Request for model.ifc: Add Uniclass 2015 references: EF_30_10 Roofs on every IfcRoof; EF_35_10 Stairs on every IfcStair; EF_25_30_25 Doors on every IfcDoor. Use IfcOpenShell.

First a look at what the model holds.

```python
import ifcopenshell

model = ifcopenshell.open("model.ifc")
print(model.schema)
print("classifications:", [c.Name for c in model.by_type("IfcClassification")])
for ifc_class in ("IfcDoor", "IfcRoof", "IfcStair", "IfcWall", "IfcWindow"):
    print(ifc_class, len(model.by_type(ifc_class)))
```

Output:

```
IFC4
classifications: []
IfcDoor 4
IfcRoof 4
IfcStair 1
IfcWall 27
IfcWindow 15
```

```python
import ifcopenshell
import ifcopenshell.api.classification

model = ifcopenshell.open("model.ifc")

system = ifcopenshell.api.classification.add_classification(model, classification="Uniclass 2015")

codes = {
    "IfcRoof": ("EF_30_10", "Roofs"),
    "IfcStair": ("EF_35_10", "Stairs"),
    "IfcDoor": ("EF_25_30_25", "Doors"),
}
for ifc_class, (code, name) in codes.items():
    products = model.by_type(ifc_class)
    ifcopenshell.api.classification.add_reference(
        model, products=products, classification=system, identification=code, name=name
    )
    print(code, len(products))

model.write("model_v2.ifc")
```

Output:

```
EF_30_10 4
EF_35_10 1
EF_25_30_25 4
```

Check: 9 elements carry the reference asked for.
